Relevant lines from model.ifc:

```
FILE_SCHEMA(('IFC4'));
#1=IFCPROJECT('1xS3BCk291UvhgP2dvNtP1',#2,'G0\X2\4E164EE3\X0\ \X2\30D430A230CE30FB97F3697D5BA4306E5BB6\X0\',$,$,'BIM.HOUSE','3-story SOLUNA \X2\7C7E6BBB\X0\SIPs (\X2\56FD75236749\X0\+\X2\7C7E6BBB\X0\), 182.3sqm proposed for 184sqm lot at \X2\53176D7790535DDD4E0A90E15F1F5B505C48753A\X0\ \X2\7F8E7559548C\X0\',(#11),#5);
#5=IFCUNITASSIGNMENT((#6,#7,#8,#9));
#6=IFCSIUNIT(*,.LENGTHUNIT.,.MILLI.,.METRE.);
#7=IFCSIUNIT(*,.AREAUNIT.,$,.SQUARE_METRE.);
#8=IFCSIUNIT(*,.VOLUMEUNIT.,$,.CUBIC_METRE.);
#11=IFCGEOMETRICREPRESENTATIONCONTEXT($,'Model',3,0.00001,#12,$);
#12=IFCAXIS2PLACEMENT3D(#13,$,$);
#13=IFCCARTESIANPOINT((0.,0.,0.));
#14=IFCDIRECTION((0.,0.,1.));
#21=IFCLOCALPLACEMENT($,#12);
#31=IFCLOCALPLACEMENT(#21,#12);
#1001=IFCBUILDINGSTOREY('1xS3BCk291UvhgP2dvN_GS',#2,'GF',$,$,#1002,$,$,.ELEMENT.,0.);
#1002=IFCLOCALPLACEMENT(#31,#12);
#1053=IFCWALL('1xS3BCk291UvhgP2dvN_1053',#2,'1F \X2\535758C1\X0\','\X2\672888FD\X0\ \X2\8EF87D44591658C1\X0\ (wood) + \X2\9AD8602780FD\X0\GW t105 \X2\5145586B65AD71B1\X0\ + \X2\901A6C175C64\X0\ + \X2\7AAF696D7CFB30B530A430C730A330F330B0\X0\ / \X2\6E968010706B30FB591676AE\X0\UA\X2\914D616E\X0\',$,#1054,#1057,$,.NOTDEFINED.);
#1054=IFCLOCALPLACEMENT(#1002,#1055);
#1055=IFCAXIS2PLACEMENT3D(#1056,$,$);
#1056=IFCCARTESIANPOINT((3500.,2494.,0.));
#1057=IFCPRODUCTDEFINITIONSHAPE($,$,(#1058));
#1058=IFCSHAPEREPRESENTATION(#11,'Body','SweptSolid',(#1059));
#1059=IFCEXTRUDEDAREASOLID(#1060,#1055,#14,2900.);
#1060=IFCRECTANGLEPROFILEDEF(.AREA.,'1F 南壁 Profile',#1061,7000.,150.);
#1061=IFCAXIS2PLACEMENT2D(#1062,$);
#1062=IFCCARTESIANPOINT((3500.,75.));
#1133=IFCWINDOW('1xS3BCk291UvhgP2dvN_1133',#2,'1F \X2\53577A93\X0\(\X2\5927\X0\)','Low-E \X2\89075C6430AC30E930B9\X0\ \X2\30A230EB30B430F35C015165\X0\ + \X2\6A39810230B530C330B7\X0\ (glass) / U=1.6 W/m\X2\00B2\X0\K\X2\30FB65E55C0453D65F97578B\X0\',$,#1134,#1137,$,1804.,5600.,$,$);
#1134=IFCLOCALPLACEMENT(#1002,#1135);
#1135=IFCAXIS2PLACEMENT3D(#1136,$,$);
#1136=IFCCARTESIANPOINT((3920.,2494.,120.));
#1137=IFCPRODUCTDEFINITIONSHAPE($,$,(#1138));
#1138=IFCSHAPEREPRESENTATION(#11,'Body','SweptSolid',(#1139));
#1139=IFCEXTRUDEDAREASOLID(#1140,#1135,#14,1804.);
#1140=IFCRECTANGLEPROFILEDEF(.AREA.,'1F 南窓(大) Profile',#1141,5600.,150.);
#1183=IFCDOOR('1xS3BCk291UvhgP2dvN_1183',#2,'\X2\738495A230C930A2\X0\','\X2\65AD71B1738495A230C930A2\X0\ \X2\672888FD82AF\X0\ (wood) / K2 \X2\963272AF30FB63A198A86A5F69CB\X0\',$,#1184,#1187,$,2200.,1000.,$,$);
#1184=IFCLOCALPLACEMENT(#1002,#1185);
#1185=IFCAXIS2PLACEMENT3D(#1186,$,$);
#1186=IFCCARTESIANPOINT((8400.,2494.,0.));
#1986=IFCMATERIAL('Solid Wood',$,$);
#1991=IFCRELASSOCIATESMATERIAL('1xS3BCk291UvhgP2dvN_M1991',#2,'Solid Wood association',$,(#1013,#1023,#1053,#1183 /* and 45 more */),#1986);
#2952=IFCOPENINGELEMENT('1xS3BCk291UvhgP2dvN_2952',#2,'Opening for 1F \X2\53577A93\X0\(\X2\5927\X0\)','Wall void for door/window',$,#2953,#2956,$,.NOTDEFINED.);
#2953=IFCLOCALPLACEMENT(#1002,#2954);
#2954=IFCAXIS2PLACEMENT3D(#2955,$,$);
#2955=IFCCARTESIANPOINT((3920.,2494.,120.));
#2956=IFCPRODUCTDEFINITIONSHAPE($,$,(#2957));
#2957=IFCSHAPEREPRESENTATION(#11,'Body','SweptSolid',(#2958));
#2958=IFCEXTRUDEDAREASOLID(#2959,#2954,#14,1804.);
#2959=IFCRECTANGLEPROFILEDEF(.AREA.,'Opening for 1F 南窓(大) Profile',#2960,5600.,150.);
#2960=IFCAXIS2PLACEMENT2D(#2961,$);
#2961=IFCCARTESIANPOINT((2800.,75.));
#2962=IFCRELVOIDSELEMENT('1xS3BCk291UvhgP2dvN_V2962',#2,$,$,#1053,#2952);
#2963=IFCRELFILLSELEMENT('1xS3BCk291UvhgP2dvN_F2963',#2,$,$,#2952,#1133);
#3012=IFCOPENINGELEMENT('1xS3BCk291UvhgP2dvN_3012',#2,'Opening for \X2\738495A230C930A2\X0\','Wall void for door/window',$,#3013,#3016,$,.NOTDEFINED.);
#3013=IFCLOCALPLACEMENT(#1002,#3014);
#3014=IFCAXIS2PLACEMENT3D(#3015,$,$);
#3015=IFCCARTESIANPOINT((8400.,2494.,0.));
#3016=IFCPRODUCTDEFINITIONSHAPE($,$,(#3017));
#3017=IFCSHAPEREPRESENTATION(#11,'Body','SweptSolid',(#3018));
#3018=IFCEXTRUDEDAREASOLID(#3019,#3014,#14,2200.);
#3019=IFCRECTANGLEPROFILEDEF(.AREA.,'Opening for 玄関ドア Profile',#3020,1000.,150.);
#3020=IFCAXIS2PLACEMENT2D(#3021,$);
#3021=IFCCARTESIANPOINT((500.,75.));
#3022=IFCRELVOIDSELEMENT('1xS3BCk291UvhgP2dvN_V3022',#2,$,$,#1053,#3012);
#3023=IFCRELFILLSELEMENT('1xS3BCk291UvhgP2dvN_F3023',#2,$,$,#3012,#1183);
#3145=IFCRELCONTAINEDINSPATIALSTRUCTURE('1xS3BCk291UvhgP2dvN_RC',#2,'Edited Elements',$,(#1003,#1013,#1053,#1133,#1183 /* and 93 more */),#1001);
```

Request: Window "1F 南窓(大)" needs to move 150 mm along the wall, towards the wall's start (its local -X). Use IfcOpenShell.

```python
import ifcopenshell
import ifcopenshell.api.geometry
import ifcopenshell.util.placement
import ifcopenshell.util.unit

model = ifcopenshell.open("model.ifc")
unit_scale = ifcopenshell.util.unit.calculate_unit_scale(model)

window = model.by_guid("1xS3BCk291UvhgP2dvN_1133")
opening = window.FillsVoids[0].RelatingOpeningElement
wall = opening.VoidsElements[0].RelatingBuildingElement

wall_matrix = ifcopenshell.util.placement.get_local_placement(wall.ObjectPlacement)
shift = wall_matrix[:3, 0] * -0.15 / unit_scale
before = ifcopenshell.util.placement.get_local_placement(window.ObjectPlacement)[:3, 3].copy()

# The window is not placed relative to its opening, so move both.
for product in (opening, window):
    matrix = ifcopenshell.util.placement.get_local_placement(product.ObjectPlacement)
    matrix[:3, 3] += shift
    ifcopenshell.api.geometry.edit_object_placement(model, product=product, matrix=matrix, is_si=False)

after = ifcopenshell.util.placement.get_local_placement(window.ObjectPlacement)[:3, 3]
print("window moved by", (after - before).round(3) + 0.0)

model.write("model-out.ifc")
```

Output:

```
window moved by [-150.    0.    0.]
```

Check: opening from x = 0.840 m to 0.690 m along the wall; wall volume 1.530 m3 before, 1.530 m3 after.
